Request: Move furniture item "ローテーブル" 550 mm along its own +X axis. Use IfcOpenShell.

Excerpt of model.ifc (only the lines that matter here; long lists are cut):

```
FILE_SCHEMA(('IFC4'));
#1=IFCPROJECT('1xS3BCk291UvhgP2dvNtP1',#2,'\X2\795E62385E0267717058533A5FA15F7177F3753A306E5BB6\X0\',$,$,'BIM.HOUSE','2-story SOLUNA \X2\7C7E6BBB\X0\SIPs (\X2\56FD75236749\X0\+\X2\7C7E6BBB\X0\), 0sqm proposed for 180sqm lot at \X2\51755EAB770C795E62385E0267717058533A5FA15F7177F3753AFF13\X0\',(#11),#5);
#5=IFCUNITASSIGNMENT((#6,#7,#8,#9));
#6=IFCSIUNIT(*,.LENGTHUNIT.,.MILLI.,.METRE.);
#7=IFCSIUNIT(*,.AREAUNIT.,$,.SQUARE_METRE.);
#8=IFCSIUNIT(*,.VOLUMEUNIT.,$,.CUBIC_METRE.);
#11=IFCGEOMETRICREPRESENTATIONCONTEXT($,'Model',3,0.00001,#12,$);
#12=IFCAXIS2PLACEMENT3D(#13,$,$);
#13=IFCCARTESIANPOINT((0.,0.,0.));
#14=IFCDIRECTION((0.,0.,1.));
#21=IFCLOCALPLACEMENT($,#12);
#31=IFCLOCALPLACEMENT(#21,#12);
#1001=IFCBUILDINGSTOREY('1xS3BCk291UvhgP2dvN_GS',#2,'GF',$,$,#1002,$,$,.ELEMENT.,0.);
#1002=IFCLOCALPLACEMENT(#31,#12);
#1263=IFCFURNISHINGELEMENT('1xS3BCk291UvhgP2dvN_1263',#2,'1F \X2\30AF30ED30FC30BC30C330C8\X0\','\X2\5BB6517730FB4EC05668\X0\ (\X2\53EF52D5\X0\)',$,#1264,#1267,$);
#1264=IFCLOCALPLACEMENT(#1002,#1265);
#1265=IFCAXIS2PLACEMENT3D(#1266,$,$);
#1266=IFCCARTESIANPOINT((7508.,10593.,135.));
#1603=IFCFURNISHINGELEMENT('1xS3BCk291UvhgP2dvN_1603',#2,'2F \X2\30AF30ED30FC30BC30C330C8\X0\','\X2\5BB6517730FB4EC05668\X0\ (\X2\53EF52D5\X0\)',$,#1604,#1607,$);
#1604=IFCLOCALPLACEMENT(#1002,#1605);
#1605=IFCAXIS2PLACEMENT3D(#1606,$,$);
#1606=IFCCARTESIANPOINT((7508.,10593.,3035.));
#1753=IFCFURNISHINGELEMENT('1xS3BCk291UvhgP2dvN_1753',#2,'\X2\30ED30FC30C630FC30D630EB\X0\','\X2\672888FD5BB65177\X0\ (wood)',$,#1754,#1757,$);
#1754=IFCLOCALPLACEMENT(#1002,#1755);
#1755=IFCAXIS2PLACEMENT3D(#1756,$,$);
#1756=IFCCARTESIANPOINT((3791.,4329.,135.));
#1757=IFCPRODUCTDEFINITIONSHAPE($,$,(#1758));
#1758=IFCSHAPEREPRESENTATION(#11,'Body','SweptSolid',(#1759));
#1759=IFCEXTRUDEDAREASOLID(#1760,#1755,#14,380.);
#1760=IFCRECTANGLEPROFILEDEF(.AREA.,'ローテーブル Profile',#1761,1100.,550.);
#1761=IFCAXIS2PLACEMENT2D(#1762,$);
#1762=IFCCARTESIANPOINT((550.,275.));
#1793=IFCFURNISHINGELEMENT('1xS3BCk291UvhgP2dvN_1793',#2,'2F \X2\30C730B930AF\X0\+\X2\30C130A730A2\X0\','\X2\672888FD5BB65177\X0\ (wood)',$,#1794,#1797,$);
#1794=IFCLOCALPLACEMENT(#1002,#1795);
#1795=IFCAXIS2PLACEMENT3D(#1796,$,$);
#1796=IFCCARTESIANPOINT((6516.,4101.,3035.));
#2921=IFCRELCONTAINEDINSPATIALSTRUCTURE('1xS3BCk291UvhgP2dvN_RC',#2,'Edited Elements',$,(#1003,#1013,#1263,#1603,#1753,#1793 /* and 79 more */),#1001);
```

```python
import ifcopenshell
import ifcopenshell.api.geometry
import ifcopenshell.util.placement

model = ifcopenshell.open("model.ifc")

item = model.by_guid("1xS3BCk291UvhgP2dvN_1753")
matrix = ifcopenshell.util.placement.get_local_placement(item.ObjectPlacement)
matrix[:3, 3] += matrix[:3, 0] * 550.0
ifcopenshell.api.geometry.edit_object_placement(model, product=item, matrix=matrix, is_si=False)

print(ifcopenshell.util.placement.get_local_placement(item.ObjectPlacement).round(3) + 0.0)

model.write("model_v2.ifc")
```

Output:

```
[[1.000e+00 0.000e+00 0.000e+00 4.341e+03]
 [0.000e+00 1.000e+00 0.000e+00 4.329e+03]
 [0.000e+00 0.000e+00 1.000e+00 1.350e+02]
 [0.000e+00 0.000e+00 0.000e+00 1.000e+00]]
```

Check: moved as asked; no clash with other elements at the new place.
